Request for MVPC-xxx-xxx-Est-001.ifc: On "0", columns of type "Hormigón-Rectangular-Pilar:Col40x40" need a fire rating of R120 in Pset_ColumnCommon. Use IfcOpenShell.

First a look at what the model holds.

```python
import ifcopenshell
import ifcopenshell.util.element

model = ifcopenshell.open("MVPC-xxx-xxx-Est-001.ifc")
print(model.schema)
storey = next(s for s in model.by_type("IfcBuildingStorey") if s.Name == "0")
columns = [e for e in ifcopenshell.util.element.get_decomposition(storey) if e.is_a("IfcColumn")]
seen = {}
for e in columns:
    element_type = ifcopenshell.util.element.get_type(e)
    key = (element_type.Name if element_type != e and element_type else None, ifcopenshell.util.element.get_pset(e, "Pset_ColumnCommon", "FireRating"))
    seen[key] = seen.get(key, 0) + 1
for (name, value), count in sorted(seen.items(), key=str):
    print(count, "x", name, "|", value)
```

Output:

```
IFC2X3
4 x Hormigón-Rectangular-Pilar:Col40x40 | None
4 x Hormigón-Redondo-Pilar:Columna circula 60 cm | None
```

```python
import ifcopenshell
import ifcopenshell.api.pset
import ifcopenshell.util.element

model = ifcopenshell.open("MVPC-xxx-xxx-Est-001.ifc")

storey = next(s for s in model.by_type("IfcBuildingStorey") if s.Name == "0")
columns = [e for e in ifcopenshell.util.element.get_decomposition(storey) if e.is_a("IfcColumn")]

count = 0
for e in columns:
    element_type = ifcopenshell.util.element.get_type(e)
    if element_type in (None, e) or element_type.Name != "Hormigón-Rectangular-Pilar:Col40x40":
        continue
    # add_pset returns the element's existing set when there is one.
    pset = ifcopenshell.api.pset.add_pset(model, product=e, name="Pset_ColumnCommon")
    ifcopenshell.api.pset.edit_pset(model, pset=pset, properties={"FireRating": "R120"})
    count += 1

print(count, "columns updated")

model.write("MVPC-xxx-xxx-Est-001-out.ifc")
```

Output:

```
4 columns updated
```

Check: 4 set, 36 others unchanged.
